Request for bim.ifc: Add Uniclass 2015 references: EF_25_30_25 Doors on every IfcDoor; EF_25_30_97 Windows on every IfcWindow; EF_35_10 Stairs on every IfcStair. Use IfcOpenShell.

First a look at what the model holds.

```python
import ifcopenshell

model = ifcopenshell.open("bim.ifc")
print(model.schema)
print("classifications:", [c.Name for c in model.by_type("IfcClassification")])
for ifc_class in ("IfcDoor", "IfcRoof", "IfcStair", "IfcWall", "IfcWindow"):
    print(ifc_class, len(model.by_type(ifc_class)))
```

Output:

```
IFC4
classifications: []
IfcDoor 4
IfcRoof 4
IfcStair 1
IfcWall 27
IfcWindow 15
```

```python
import ifcopenshell
import ifcopenshell.api.classification

model = ifcopenshell.open("bim.ifc")

system = ifcopenshell.api.classification.add_classification(model, classification="Uniclass 2015")

codes = {
    "IfcDoor": ("EF_25_30_25", "Doors"),
    "IfcWindow": ("EF_25_30_97", "Windows"),
    "IfcStair": ("EF_35_10", "Stairs"),
}
for ifc_class, (code, name) in codes.items():
    products = model.by_type(ifc_class)
    ifcopenshell.api.classification.add_reference(
        model, products=products, classification=system, identification=code, name=name
    )
    print(code, len(products))

model.write("bim_v2.ifc")
```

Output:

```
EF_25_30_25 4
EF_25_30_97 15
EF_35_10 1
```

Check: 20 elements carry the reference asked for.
